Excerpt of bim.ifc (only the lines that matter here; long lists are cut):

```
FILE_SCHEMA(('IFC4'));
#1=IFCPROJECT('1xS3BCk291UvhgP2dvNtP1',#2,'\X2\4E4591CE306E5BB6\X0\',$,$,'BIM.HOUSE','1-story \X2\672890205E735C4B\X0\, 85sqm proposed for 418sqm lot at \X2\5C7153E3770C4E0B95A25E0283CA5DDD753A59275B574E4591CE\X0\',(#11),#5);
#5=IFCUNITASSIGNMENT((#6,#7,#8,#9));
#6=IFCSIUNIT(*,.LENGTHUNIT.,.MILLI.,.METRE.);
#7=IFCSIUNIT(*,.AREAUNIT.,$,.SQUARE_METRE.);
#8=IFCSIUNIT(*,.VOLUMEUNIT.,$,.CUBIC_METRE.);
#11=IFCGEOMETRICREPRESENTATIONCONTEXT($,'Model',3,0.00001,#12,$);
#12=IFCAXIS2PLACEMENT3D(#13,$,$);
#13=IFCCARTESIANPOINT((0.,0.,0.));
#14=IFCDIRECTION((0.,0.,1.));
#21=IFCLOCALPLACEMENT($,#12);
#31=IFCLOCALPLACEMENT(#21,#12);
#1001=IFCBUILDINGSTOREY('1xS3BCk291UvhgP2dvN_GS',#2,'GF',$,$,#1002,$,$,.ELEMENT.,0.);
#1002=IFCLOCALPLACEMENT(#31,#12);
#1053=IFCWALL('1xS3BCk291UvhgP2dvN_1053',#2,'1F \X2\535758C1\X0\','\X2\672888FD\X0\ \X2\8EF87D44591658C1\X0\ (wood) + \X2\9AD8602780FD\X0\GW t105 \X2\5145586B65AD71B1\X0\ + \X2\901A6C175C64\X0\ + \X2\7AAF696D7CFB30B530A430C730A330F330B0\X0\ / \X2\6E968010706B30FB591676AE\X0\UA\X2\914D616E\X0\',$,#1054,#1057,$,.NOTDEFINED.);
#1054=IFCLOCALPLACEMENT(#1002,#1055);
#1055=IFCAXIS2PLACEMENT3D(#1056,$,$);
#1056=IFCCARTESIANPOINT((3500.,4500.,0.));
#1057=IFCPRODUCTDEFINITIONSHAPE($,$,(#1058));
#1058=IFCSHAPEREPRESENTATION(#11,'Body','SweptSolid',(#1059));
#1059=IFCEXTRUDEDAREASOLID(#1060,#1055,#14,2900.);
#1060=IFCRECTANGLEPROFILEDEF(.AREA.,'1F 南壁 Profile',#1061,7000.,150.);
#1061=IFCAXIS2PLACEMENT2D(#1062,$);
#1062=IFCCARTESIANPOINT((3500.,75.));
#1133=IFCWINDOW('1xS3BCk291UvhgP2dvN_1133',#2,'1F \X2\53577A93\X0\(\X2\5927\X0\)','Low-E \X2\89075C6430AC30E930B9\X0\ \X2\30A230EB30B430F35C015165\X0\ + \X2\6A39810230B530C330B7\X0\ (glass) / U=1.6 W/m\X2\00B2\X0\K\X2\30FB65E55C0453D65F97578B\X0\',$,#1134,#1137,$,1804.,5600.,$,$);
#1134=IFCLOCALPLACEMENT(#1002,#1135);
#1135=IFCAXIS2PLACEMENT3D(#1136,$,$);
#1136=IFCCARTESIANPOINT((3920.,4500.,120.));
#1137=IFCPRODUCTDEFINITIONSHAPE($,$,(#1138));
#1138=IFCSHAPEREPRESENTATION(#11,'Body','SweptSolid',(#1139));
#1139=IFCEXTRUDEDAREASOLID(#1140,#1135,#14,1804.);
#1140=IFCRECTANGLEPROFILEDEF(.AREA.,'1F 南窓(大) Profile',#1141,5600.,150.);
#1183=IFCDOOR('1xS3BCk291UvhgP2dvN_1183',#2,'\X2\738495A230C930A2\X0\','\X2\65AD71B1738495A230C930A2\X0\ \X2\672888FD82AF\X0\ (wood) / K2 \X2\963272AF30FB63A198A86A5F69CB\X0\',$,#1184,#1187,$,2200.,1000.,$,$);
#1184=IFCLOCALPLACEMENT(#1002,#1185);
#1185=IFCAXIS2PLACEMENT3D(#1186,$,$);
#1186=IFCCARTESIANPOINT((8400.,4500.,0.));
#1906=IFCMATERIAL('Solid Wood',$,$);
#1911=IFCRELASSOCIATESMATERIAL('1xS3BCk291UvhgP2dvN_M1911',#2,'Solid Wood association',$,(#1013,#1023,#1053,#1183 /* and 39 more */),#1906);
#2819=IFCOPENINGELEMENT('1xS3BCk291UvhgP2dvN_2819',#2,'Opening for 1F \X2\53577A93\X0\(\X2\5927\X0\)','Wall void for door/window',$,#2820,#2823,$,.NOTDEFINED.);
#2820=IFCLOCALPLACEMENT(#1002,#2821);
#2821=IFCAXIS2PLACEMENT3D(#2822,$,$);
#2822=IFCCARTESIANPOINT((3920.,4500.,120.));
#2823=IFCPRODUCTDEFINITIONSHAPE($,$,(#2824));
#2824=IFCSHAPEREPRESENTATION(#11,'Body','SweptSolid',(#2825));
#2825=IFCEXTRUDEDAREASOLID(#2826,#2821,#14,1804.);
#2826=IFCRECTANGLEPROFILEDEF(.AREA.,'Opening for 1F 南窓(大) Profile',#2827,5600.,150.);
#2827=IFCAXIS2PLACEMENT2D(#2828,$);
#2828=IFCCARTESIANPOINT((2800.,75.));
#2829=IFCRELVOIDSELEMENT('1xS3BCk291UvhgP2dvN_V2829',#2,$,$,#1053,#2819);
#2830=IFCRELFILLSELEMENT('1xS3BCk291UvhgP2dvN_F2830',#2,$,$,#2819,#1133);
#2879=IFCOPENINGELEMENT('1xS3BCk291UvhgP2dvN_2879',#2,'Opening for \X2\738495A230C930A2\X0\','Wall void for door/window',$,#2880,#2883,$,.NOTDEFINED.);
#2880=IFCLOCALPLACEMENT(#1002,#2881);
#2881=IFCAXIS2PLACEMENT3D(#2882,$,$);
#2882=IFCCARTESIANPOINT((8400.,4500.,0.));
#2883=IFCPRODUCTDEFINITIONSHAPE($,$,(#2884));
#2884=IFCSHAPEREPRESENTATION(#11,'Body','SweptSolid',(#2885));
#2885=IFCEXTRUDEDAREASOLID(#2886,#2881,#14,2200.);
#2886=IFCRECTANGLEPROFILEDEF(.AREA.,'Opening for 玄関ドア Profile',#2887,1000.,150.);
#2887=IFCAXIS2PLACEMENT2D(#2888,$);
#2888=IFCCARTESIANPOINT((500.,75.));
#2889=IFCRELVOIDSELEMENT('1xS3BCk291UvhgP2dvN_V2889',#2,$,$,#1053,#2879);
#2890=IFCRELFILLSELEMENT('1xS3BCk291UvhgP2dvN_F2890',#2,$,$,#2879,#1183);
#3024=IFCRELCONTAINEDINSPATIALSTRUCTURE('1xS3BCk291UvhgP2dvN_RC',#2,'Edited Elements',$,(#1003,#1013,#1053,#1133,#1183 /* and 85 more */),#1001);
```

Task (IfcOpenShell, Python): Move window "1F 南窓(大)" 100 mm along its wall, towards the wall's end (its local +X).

```python
import ifcopenshell
import ifcopenshell.api.geometry
import ifcopenshell.util.placement

model = ifcopenshell.open("bim.ifc")

window = model.by_id(1133)
opening = window.FillsVoids[0].RelatingOpeningElement
wall = opening.VoidsElements[0].RelatingBuildingElement

wall_matrix = ifcopenshell.util.placement.get_local_placement(wall.ObjectPlacement)
shift = wall_matrix[:3, 0] * 100.0
before = ifcopenshell.util.placement.get_local_placement(window.ObjectPlacement)[:3, 3].copy()

# The window is not placed relative to its opening, so move both.
for product in (opening, window):
    matrix = ifcopenshell.util.placement.get_local_placement(product.ObjectPlacement)
    matrix[:3, 3] += shift
    ifcopenshell.api.geometry.edit_object_placement(model, product=product, matrix=matrix, is_si=False)

after = ifcopenshell.util.placement.get_local_placement(window.ObjectPlacement)[:3, 3]
print("window moved by", (after - before).round(3) + 0.0)

model.write("bim_updated.ifc")
```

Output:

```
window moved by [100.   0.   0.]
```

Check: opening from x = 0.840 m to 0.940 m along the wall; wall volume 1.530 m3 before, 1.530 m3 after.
